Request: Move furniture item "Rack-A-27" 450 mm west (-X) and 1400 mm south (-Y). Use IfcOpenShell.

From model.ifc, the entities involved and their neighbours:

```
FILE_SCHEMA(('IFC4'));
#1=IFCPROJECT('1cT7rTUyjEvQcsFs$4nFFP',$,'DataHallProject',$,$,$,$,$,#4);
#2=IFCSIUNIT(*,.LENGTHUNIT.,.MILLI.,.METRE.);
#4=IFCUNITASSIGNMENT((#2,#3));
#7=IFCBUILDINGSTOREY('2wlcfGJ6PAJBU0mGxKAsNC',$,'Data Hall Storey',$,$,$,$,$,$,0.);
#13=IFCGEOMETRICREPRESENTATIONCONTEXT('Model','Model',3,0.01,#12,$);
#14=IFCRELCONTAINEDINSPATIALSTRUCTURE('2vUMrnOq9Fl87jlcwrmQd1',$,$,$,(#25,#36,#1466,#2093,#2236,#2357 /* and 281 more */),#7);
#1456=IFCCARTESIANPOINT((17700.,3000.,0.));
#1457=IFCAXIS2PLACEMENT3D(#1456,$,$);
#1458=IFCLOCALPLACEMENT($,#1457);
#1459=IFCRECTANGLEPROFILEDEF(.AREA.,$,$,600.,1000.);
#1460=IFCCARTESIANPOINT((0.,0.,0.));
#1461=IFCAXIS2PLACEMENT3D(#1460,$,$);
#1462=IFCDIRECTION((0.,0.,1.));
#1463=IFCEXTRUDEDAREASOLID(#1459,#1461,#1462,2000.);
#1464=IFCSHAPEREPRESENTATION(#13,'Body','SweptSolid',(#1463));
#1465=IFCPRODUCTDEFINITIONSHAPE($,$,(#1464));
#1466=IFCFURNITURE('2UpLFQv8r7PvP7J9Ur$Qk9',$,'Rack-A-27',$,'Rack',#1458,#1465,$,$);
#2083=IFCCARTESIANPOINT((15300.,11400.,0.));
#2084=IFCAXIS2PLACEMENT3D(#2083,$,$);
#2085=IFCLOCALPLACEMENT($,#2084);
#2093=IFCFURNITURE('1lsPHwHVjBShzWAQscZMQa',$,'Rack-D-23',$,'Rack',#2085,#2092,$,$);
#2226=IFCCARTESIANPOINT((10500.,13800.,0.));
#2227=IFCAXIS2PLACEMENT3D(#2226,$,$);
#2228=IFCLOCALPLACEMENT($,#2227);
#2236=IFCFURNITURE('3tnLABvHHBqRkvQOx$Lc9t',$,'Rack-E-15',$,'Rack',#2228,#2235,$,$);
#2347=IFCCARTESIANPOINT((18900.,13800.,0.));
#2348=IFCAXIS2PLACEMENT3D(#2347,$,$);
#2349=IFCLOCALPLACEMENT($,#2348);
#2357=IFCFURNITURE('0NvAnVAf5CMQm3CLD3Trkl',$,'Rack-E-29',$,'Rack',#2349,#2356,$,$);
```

```python
import ifcopenshell
import ifcopenshell.api.geometry
import ifcopenshell.util.placement
import ifcopenshell.util.unit

model = ifcopenshell.open("model.ifc")
unit_scale = ifcopenshell.util.unit.calculate_unit_scale(model)

item = model.by_guid("2UpLFQv8r7PvP7J9Ur$Qk9")
matrix = ifcopenshell.util.placement.get_local_placement(item.ObjectPlacement)
matrix[0, 3] -= 0.45 / unit_scale
matrix[1, 3] -= 1.4 / unit_scale
ifcopenshell.api.geometry.edit_object_placement(model, product=item, matrix=matrix, is_si=False)

print(ifcopenshell.util.placement.get_local_placement(item.ObjectPlacement).round(3) + 0.0)

model.write("model_v2.ifc")
```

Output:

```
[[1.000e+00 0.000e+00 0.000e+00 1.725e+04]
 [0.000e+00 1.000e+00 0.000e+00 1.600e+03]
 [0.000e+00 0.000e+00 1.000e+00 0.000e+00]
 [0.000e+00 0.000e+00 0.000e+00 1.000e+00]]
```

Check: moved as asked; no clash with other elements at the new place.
